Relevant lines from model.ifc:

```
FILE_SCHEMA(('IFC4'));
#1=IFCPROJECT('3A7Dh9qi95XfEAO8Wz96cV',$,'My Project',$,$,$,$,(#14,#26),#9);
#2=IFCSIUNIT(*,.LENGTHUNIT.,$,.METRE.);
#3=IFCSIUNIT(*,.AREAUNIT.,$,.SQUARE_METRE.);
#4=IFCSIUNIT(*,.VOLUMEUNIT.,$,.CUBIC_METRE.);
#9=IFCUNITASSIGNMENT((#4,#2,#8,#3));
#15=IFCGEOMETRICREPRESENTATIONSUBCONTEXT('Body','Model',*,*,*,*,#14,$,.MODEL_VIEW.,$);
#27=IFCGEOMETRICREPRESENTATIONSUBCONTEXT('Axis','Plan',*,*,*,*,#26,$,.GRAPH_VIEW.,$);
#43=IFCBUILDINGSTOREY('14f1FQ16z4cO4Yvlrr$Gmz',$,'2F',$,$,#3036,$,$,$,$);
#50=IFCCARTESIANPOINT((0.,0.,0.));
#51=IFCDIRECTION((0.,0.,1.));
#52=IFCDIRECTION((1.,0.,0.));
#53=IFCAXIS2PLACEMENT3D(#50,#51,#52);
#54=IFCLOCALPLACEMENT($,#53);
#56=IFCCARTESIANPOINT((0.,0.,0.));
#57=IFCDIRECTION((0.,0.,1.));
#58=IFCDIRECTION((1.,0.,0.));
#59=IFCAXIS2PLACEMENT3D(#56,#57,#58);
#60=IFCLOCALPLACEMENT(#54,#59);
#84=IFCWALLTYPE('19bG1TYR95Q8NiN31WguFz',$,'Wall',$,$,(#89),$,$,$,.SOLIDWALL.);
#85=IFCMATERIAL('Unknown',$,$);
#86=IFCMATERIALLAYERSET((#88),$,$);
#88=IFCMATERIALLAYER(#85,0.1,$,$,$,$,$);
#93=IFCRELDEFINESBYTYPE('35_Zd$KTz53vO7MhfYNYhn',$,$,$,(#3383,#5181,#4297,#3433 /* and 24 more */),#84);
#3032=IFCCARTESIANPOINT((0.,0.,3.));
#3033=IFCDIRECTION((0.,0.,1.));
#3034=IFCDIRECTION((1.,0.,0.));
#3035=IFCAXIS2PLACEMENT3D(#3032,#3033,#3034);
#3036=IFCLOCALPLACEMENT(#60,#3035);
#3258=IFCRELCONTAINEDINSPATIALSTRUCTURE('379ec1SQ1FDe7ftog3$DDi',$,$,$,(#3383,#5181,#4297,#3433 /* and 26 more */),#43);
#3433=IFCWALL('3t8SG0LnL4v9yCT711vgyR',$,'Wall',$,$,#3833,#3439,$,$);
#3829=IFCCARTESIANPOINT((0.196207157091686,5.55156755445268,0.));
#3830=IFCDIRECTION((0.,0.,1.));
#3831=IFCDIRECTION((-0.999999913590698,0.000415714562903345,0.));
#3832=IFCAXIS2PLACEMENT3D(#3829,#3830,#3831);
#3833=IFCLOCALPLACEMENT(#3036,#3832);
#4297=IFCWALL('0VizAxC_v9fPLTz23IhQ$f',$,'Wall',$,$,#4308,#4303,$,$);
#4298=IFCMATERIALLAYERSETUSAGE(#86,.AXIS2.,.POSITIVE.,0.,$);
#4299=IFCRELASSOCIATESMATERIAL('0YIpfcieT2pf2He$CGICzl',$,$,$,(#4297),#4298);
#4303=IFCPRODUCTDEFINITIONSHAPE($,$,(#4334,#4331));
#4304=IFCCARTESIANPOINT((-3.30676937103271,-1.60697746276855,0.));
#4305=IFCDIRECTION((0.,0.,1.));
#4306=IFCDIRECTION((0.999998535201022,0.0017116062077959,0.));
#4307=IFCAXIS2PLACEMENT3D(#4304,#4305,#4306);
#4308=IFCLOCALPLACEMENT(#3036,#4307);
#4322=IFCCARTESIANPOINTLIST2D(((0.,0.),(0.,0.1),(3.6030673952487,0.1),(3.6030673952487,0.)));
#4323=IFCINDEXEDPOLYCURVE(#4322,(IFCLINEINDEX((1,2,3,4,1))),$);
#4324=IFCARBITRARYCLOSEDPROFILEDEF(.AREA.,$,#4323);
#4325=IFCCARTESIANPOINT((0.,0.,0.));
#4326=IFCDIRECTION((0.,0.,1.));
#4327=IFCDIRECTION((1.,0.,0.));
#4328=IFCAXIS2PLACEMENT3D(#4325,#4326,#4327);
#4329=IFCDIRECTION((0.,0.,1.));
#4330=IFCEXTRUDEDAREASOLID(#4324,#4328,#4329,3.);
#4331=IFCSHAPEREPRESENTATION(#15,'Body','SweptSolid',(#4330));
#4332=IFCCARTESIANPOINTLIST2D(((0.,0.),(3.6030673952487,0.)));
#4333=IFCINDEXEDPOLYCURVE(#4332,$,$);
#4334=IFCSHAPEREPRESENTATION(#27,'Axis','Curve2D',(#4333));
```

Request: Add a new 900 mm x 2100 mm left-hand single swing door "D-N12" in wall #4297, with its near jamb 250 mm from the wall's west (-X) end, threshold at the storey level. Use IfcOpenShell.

```python
import numpy as np
import ifcopenshell
import ifcopenshell.api.feature
import ifcopenshell.api.geometry
import ifcopenshell.api.root
import ifcopenshell.api.spatial
import ifcopenshell.geom
import ifcopenshell.util.element
import ifcopenshell.util.placement
import ifcopenshell.util.representation
import ifcopenshell.util.shape
import ifcopenshell.util.unit

model = ifcopenshell.open("model.ifc")
unit_scale = ifcopenshell.util.unit.calculate_unit_scale(model)
settings = ifcopenshell.geom.settings()


def volume(element):
    """Net volume in cubic metres, openings subtracted."""
    shape = ifcopenshell.geom.create_shape(settings, element)
    return ifcopenshell.util.shape.get_volume(shape.geometry)


wall = model.by_id(4297)
storey = ifcopenshell.util.element.get_container(wall, ifc_class="IfcBuildingStorey")
context = ifcopenshell.util.representation.get_context(model, "Model", "Body", "MODEL_VIEW")
before = volume(wall)

width, height, from_end, sill = 0.9, 2.1, 0.25, 0.0  # metres

# The wall runs along its own X axis, and the end named is its -X end.
wall_shape = ifcopenshell.geom.create_shape(settings, wall)
x, y, z = ifcopenshell.util.shape.get_vertices(wall_shape.geometry).T
start = x.min() + from_end
face, thickness = float(y.min()), float(y.max() - y.min())
wall_matrix = ifcopenshell.util.placement.get_local_placement(wall.ObjectPlacement)
level = ifcopenshell.util.placement.get_local_placement(storey.ObjectPlacement)[2, 3]


def in_wall(x, y):
    """Placement at x, y metres in the wall's axes, at sill height."""
    matrix = wall_matrix.copy()
    matrix[:, 3] = wall_matrix @ np.array([x / unit_scale, y / unit_scale, 0.0, 1.0])
    matrix[2, 3] = level + sill / unit_scale
    return matrix


# Opening: a box that overshoots both wall faces by 50 mm.
opening = ifcopenshell.api.root.create_entity(model, ifc_class="IfcOpeningElement", predefined_type="OPENING")
box = ifcopenshell.api.geometry.add_wall_representation(
    model, context=context, length=width, height=height, thickness=thickness + 0.1
)
ifcopenshell.api.geometry.assign_representation(model, product=opening, representation=box)
ifcopenshell.api.geometry.edit_object_placement(model, product=opening, matrix=in_wall(start, face - 0.05), is_si=False)
ifcopenshell.api.feature.add_feature(model, feature=opening, element=wall)

door = ifcopenshell.api.root.create_entity(model, ifc_class="IfcDoor", name="D-N12", predefined_type="DOOR")
door.OverallWidth, door.OverallHeight = width / unit_scale, height / unit_scale
door.OperationType = "SINGLE_SWING_LEFT"
body = ifcopenshell.api.geometry.add_door_representation(
    model,
    context=context,
    overall_width=door.OverallWidth,
    overall_height=door.OverallHeight,
    operation_type="SINGLE_SWING_LEFT",
    lining_properties={"LiningDepth": thickness / unit_scale, "ThresholdDepth": thickness / unit_scale},
)
ifcopenshell.api.geometry.assign_representation(model, product=door, representation=body)
ifcopenshell.api.spatial.assign_container(model, products=[door], relating_structure=storey)
ifcopenshell.api.feature.add_filling(model, opening=opening, element=door)

# The lining spans the wall, so the door starts at the wall face.
ifcopenshell.api.geometry.edit_object_placement(model, product=door, matrix=in_wall(start, face), is_si=False)

after = volume(wall)

print(f"wall volume {before:.3f} -> {after:.3f} m3")

model.write("model_updated.ifc")
```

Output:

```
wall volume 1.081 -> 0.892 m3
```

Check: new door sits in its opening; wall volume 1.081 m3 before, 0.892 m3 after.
